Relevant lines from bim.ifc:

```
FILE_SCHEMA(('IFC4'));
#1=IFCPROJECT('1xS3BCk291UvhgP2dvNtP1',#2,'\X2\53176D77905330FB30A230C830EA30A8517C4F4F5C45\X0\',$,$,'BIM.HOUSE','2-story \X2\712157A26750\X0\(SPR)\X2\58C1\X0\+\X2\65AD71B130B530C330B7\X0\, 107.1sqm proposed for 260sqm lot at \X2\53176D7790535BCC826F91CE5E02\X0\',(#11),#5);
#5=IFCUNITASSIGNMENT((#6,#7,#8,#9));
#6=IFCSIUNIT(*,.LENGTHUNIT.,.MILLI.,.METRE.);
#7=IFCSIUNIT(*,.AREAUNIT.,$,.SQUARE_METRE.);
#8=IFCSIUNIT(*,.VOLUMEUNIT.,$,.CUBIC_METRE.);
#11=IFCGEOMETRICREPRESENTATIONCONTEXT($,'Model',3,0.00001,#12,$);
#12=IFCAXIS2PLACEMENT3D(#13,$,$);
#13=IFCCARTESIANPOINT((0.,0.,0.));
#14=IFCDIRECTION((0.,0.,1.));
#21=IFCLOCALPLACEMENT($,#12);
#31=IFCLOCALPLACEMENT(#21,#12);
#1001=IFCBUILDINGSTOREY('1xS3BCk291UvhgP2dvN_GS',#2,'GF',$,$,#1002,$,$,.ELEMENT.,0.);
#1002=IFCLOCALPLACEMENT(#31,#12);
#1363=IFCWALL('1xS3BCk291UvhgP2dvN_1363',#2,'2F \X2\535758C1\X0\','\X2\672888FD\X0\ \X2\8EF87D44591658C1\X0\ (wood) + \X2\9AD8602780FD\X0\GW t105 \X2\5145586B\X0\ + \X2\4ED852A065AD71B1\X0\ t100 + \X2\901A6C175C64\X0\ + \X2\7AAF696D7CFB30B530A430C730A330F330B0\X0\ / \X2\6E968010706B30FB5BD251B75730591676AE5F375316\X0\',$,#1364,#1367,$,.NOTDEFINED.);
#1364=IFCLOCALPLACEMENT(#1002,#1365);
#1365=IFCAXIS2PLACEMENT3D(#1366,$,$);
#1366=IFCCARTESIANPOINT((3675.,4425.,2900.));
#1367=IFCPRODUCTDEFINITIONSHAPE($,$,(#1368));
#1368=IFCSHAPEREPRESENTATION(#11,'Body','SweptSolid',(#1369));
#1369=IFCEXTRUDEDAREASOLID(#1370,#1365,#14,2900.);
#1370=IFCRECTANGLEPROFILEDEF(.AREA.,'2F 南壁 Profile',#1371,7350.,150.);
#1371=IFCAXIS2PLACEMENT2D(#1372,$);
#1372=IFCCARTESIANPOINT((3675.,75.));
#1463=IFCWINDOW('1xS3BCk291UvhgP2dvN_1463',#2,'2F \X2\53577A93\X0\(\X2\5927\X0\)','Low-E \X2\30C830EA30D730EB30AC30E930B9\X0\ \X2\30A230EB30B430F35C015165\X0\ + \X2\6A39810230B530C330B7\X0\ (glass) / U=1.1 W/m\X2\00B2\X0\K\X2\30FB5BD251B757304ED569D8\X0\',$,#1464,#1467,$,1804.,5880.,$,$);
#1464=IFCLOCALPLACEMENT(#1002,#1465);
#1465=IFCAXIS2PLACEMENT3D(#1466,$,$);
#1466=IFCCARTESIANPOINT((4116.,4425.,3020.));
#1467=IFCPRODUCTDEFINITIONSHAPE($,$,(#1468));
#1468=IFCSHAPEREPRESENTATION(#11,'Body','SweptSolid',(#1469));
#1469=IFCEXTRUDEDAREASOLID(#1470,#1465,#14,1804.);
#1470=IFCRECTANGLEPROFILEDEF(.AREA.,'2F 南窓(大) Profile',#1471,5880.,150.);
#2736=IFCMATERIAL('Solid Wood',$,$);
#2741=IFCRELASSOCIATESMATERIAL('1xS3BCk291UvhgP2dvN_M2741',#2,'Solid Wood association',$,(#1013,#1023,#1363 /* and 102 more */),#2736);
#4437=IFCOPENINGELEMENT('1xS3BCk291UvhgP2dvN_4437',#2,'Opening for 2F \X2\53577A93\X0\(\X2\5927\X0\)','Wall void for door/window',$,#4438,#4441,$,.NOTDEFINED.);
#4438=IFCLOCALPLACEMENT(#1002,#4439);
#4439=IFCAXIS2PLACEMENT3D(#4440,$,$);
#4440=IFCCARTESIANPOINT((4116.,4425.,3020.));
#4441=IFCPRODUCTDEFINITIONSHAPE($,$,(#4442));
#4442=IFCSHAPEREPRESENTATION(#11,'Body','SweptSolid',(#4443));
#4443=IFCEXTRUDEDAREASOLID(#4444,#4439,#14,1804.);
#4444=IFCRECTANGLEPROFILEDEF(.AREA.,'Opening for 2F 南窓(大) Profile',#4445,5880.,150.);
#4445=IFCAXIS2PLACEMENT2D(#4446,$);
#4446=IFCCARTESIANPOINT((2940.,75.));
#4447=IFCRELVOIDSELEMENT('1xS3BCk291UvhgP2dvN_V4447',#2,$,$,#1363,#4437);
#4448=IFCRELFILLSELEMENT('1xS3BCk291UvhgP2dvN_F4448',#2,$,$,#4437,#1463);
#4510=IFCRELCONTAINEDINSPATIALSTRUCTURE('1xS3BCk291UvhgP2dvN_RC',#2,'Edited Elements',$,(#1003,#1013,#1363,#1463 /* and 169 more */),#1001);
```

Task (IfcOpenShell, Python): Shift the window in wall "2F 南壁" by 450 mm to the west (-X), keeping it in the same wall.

```python
import ifcopenshell
import ifcopenshell.api.geometry
import ifcopenshell.util.placement

model = ifcopenshell.open("bim.ifc")

window = model.by_guid("1xS3BCk291UvhgP2dvN_1463")
opening = window.FillsVoids[0].RelatingOpeningElement
wall = opening.VoidsElements[0].RelatingBuildingElement

wall_matrix = ifcopenshell.util.placement.get_local_placement(wall.ObjectPlacement)
shift = wall_matrix[:3, 0] * -450.0
before = ifcopenshell.util.placement.get_local_placement(window.ObjectPlacement)[:3, 3].copy()

# The window is not placed relative to its opening, so move both.
for product in (opening, window):
    matrix = ifcopenshell.util.placement.get_local_placement(product.ObjectPlacement)
    matrix[:3, 3] += shift
    ifcopenshell.api.geometry.edit_object_placement(model, product=product, matrix=matrix, is_si=False)

after = ifcopenshell.util.placement.get_local_placement(window.ObjectPlacement)[:3, 3]
print("window moved by", (after - before).round(3) + 0.0)

model.write("bim_edited.ifc")
```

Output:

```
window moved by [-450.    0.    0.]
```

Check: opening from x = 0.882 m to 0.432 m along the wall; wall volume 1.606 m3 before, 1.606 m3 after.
